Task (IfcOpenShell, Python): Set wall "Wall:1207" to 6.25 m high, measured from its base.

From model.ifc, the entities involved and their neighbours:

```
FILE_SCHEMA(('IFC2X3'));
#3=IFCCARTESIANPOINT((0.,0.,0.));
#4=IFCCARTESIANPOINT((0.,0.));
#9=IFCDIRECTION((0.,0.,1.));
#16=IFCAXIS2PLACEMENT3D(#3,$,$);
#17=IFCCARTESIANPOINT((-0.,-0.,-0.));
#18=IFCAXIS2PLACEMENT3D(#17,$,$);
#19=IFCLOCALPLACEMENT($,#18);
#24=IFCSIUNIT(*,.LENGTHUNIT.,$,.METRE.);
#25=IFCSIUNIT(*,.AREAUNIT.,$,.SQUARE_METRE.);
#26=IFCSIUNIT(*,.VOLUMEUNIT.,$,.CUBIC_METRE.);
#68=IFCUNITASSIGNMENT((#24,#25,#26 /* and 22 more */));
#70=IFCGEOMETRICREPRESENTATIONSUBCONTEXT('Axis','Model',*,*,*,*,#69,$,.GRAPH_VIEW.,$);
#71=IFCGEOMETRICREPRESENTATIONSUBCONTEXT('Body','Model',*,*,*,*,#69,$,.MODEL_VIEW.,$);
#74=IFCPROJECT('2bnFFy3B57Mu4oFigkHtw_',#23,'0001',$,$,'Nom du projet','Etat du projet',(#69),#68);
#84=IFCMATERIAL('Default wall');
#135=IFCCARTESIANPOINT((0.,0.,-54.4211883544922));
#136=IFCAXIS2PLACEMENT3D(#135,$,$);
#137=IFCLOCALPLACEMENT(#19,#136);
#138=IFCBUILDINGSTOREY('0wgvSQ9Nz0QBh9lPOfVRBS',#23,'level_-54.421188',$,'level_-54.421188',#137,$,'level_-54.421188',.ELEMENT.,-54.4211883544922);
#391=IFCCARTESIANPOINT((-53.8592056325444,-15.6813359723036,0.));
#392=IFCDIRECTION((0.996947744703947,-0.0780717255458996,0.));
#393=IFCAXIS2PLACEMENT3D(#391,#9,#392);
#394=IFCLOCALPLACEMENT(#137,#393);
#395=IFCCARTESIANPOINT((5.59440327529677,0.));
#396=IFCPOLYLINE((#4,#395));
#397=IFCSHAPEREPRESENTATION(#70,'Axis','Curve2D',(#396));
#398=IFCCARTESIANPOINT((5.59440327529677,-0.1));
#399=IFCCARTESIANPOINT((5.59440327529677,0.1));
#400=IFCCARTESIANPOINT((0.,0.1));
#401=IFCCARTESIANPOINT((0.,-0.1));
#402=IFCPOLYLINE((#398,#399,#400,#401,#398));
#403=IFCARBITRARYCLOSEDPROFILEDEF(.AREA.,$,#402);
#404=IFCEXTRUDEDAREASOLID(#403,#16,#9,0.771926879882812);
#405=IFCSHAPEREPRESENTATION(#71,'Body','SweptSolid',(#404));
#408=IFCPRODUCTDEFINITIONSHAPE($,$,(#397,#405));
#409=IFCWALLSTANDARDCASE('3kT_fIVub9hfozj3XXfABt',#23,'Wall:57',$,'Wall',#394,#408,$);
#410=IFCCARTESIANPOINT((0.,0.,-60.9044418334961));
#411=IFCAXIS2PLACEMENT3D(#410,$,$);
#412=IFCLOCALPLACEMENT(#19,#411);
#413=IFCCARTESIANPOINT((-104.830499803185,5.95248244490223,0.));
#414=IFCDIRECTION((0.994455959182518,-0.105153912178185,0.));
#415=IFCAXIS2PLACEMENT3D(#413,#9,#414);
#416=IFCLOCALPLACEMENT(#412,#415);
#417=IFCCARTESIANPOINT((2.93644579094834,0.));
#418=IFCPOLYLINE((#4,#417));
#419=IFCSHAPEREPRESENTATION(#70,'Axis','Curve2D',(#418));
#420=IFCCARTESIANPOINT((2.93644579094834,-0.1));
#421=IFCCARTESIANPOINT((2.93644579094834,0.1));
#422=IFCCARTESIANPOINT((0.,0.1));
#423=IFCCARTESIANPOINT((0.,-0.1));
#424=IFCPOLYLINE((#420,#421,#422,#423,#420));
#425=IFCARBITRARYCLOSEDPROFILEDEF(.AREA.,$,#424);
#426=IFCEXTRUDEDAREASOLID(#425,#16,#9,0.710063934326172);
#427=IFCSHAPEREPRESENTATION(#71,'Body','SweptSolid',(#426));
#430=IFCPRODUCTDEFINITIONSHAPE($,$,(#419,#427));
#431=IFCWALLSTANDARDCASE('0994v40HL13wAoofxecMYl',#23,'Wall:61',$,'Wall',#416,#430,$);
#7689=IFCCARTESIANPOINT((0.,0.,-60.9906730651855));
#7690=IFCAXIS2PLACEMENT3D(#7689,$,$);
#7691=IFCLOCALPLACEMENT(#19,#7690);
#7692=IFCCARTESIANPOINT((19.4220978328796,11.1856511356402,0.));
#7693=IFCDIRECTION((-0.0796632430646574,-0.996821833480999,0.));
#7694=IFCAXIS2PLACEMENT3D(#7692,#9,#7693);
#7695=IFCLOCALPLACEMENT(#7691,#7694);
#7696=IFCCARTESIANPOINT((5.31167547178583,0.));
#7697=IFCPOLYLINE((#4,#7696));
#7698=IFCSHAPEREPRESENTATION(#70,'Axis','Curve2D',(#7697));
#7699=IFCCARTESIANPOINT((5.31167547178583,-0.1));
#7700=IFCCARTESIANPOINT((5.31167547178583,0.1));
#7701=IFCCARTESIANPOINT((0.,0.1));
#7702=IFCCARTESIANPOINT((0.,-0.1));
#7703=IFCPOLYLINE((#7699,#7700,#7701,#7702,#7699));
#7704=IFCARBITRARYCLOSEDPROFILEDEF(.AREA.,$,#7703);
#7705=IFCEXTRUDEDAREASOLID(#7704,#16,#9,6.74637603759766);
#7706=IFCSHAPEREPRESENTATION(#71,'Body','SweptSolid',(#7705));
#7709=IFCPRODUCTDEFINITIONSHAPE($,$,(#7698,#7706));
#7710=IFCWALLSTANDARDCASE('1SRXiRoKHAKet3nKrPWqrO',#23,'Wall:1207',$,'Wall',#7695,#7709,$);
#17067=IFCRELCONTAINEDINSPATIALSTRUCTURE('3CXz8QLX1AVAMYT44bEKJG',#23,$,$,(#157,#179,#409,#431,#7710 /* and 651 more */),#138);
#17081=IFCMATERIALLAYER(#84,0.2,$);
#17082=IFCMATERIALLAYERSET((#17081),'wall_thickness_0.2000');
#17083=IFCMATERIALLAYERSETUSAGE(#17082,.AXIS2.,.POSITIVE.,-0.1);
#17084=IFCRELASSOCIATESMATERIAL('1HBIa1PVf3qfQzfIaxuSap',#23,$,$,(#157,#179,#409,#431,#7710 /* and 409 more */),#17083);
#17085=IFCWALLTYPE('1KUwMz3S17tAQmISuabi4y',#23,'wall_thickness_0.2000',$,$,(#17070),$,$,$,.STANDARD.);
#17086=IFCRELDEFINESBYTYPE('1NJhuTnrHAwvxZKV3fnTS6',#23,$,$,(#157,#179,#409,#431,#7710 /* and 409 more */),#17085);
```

```python
import ifcopenshell
import ifcopenshell.geom
import ifcopenshell.util.representation
import ifcopenshell.util.shape

model = ifcopenshell.open("model.ifc")
settings = ifcopenshell.geom.settings()


def volume(element):
    """Net volume in cubic metres, openings subtracted."""
    shape = ifcopenshell.geom.create_shape(settings, element)
    return ifcopenshell.util.shape.get_volume(shape.geometry)


wall = model.by_id(7710)
before = volume(wall)

body = ifcopenshell.util.representation.get_representation(wall, "Model", "Body")
solid = body.Items[0]
old_height = solid.Depth
solid.Depth = 6.25
after = volume(wall)

print(f"height {old_height:g} -> {solid.Depth:g}, volume {before:.3f} -> {after:.3f} m3")

model.write("model_rev.ifc")
```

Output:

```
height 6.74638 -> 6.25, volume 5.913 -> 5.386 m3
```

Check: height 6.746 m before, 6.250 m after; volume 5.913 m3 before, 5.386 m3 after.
